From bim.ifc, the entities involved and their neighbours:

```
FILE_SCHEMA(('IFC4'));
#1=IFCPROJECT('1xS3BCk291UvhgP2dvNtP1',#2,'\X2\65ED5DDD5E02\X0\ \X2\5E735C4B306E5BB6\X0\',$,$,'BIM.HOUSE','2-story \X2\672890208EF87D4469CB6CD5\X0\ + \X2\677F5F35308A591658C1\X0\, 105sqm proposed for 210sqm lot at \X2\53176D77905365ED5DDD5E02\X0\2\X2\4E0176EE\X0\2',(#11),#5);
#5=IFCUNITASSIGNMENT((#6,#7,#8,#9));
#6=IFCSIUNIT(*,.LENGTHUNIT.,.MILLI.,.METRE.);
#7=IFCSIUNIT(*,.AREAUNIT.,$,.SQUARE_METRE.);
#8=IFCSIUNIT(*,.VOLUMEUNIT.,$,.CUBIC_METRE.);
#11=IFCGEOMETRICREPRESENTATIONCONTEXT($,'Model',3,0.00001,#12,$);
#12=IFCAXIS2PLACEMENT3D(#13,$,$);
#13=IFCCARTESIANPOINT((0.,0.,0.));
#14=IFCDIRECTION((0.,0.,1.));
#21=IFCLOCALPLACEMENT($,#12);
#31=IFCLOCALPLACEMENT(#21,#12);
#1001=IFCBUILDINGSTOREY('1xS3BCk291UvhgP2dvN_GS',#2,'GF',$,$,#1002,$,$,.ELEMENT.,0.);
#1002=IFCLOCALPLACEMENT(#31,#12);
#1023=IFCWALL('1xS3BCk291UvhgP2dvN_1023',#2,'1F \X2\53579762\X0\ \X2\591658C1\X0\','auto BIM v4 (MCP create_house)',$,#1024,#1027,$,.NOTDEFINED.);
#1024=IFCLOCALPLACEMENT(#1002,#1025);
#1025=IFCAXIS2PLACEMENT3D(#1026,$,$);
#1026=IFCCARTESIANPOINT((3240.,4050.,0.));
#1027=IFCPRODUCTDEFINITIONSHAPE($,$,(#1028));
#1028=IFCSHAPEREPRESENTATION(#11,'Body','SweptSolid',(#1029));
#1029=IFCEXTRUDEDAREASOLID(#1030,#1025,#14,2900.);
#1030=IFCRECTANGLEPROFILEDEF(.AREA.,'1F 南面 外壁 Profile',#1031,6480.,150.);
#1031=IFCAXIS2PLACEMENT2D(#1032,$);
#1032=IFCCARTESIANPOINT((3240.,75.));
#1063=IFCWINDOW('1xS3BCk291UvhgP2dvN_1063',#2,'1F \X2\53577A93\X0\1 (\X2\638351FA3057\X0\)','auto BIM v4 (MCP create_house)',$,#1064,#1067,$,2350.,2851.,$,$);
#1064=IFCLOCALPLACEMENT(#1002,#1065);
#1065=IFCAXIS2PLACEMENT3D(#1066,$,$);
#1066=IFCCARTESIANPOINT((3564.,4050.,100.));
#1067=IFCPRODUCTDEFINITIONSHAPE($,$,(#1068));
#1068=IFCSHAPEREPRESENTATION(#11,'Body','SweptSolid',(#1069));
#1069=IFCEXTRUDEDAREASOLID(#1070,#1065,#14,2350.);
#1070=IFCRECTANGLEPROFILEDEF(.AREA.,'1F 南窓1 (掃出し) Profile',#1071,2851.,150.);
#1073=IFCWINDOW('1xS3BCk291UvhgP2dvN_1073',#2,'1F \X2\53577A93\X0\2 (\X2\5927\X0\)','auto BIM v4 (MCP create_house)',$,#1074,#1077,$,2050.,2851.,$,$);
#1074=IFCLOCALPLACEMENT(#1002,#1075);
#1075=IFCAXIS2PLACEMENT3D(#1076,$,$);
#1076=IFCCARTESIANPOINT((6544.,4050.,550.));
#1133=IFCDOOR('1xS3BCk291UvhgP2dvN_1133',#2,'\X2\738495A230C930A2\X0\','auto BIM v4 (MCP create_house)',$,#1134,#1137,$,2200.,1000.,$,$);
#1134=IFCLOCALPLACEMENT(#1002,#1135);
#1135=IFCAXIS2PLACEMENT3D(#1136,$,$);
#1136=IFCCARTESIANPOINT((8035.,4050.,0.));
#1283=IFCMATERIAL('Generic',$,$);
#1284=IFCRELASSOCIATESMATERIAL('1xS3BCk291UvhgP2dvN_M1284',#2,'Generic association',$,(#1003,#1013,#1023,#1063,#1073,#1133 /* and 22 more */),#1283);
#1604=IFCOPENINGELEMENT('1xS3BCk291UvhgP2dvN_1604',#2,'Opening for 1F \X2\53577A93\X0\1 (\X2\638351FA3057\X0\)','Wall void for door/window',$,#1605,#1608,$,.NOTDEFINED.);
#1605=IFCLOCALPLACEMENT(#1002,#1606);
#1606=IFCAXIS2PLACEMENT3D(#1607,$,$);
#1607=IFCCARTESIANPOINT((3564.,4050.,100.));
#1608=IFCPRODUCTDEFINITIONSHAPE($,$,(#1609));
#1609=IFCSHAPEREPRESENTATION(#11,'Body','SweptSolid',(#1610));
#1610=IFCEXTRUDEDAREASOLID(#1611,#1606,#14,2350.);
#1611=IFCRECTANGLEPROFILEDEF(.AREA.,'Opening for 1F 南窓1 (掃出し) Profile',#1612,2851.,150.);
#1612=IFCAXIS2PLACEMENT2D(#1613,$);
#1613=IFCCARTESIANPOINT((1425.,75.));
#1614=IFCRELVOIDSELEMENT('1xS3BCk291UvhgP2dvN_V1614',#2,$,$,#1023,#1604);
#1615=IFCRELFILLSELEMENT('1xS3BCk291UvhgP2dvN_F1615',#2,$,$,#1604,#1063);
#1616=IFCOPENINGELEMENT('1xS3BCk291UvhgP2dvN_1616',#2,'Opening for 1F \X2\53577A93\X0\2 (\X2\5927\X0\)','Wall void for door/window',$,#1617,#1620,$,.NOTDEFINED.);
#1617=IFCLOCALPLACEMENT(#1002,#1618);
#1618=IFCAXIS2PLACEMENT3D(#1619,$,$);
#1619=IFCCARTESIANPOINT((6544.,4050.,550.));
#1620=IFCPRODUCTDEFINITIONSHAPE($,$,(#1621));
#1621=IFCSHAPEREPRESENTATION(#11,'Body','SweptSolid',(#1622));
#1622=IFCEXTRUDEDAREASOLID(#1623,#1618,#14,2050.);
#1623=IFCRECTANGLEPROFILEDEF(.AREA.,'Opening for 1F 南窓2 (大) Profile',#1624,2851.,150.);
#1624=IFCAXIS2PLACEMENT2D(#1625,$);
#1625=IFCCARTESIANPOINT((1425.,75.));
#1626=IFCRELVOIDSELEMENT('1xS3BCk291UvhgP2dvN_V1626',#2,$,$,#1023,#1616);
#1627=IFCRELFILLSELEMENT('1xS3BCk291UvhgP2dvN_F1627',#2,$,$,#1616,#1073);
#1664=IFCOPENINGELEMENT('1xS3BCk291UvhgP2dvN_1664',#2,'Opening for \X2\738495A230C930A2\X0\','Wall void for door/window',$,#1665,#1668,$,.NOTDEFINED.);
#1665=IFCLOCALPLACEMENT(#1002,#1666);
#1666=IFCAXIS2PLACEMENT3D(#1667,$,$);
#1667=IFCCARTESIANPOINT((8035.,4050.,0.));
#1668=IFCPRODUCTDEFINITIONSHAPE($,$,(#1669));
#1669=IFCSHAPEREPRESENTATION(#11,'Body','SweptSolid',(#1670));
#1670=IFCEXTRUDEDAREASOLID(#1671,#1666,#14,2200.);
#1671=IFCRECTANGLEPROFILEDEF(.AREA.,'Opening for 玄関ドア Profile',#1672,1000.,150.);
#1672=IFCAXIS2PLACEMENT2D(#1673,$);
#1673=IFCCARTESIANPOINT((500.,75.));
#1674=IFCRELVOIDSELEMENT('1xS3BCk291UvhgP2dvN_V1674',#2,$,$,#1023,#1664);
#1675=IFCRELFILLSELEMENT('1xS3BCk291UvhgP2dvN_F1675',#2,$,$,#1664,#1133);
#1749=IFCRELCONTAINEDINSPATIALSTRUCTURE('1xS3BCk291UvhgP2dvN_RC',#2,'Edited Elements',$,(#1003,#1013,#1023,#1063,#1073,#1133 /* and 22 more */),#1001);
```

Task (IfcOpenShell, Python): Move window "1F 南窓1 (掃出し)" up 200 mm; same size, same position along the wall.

```python
import numpy as np
import ifcopenshell
import ifcopenshell.api.geometry
import ifcopenshell.util.placement
import ifcopenshell.util.unit

model = ifcopenshell.open("bim.ifc")
unit_scale = ifcopenshell.util.unit.calculate_unit_scale(model)

window = model.by_guid("1xS3BCk291UvhgP2dvN_1063")
opening = window.FillsVoids[0].RelatingOpeningElement
dz = 200.0

shift = np.array([0.0, 0.0, dz])
# The window is not placed relative to its opening, so move both.
for product in (opening, window):
    matrix = ifcopenshell.util.placement.get_local_placement(product.ObjectPlacement)
    matrix[:3, 3] += shift
    ifcopenshell.api.geometry.edit_object_placement(model, product=product, matrix=matrix, is_si=False)

print(f"moved by {dz * unit_scale:+.3f} m")

model.write("bim_edited.ifc")
```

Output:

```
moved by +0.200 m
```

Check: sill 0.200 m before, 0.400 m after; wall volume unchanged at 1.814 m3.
